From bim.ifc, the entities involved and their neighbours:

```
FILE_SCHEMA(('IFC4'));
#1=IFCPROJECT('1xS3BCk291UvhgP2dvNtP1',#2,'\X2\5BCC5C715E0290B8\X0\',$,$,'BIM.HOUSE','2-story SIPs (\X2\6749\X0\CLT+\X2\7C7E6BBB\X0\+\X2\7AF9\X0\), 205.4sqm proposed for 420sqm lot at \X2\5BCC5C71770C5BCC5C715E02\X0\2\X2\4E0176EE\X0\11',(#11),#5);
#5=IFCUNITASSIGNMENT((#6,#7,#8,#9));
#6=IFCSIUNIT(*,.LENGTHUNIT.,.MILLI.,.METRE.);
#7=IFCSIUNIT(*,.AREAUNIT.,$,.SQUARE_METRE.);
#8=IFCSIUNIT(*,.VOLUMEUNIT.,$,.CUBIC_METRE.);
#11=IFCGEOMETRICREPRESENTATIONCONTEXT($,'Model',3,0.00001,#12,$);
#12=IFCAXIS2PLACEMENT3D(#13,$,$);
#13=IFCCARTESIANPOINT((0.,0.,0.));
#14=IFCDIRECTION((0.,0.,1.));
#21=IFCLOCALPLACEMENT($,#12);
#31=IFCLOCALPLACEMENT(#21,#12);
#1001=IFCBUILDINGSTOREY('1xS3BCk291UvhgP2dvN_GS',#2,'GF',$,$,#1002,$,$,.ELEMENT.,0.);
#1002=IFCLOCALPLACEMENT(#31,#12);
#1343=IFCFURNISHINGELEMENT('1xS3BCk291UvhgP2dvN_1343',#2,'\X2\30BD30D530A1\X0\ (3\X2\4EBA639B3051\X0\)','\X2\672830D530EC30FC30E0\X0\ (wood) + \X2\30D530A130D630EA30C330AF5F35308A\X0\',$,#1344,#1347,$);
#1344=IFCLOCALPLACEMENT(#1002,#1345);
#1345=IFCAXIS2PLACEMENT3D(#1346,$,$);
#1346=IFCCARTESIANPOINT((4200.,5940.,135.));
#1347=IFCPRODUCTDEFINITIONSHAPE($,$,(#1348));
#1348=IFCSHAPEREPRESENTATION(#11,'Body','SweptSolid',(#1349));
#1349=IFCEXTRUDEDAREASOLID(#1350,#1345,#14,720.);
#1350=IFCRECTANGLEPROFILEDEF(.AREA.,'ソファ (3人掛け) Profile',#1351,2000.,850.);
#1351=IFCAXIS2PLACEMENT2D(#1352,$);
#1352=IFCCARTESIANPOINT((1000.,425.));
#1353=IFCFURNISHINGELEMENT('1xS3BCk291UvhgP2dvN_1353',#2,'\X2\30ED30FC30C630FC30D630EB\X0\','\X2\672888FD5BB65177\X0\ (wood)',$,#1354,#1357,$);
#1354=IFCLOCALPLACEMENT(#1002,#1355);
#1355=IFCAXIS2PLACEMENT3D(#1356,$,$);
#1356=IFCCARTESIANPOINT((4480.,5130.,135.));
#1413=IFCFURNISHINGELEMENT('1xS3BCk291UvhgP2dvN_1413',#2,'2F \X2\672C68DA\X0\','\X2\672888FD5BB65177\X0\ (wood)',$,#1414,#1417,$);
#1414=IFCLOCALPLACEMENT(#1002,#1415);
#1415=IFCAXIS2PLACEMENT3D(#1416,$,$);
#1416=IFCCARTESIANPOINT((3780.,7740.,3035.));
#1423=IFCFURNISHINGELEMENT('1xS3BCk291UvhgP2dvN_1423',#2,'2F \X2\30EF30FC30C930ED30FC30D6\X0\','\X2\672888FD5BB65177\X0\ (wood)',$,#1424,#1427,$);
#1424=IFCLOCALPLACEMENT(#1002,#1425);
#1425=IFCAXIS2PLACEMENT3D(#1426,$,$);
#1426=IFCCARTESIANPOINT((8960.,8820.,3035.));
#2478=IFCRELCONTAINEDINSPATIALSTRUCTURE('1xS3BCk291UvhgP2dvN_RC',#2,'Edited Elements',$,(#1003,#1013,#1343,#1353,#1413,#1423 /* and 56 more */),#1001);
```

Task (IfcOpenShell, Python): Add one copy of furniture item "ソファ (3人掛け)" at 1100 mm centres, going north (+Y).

```python
import numpy as np
import ifcopenshell
import ifcopenshell.api.geometry
import ifcopenshell.api.root
import ifcopenshell.util.element
import ifcopenshell.util.placement

model = ifcopenshell.open("bim.ifc")


def reuse_history(source, copy):
    """copy_class also copies each property set's owner history, people and application; keep the originals."""
    for rel in copy.IsDefinedBy:
        if rel.is_a("IfcRelDefinesByProperties") and (history := rel.RelatingPropertyDefinition.OwnerHistory):
            rel.RelatingPropertyDefinition.OwnerHistory = source.OwnerHistory
            ifcopenshell.util.element.remove_deep2(model, history)


source = model.by_guid("1xS3BCk291UvhgP2dvN_1343")
base = ifcopenshell.util.placement.get_local_placement(source.ObjectPlacement)
step = np.array([0.0, 1.0, 0.0]) * 1100.0

for i in range(1, 2):
    copy = ifcopenshell.api.root.copy_class(model, product=source)
    copy.Representation = ifcopenshell.util.element.copy_deep(
        model, source.Representation, exclude=["IfcGeometricRepresentationContext", "IfcRepresentationMap"]
    )
    reuse_history(source, copy)
    matrix = base.copy()
    matrix[:3, 3] += i * step
    print("added at", matrix[:3, 3].round(3) + 0.0)
    ifcopenshell.api.geometry.edit_object_placement(model, product=copy, matrix=matrix, is_si=False)

model.write("bim-out.ifc")
```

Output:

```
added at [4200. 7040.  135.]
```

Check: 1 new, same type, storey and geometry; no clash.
